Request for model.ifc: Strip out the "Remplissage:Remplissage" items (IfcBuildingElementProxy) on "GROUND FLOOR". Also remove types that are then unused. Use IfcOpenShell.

First a look at what the model holds.

```python
import ifcopenshell
import ifcopenshell.util.element

model = ifcopenshell.open("model.ifc")
print(model.schema)
storey = next(s for s in model.by_type("IfcBuildingStorey") if s.Name == "GROUND FLOOR")
proxies = [e for e in ifcopenshell.util.element.get_decomposition(storey) if e.is_a("IfcBuildingElementProxy")]
seen = {}
for e in proxies:
    element_type = ifcopenshell.util.element.get_type(e)
    name = element_type.Name if element_type not in (None, e) else None
    seen[name] = seen.get(name, 0) + 1
for name, count in sorted(seen.items(), key=str):
    print(count, "x", name)
```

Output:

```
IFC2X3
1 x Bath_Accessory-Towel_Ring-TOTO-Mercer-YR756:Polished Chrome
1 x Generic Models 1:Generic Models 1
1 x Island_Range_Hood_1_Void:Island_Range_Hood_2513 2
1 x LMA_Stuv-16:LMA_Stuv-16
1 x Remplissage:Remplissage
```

```python
import ifcopenshell
import ifcopenshell.api.root
import ifcopenshell.util.element

model = ifcopenshell.open("model.ifc")

storey = next(s for s in model.by_type("IfcBuildingStorey") if s.Name == "GROUND FLOOR")
proxies = [e for e in ifcopenshell.util.element.get_decomposition(storey) if e.is_a("IfcBuildingElementProxy")]
targets = [e for e in proxies if (t := ifcopenshell.util.element.get_type(e)) not in (None, e) and t.Name == "Remplissage:Remplissage"]
types = {ifcopenshell.util.element.get_type(e) for e in targets} - {None, *targets}

for e in targets:
    ifcopenshell.api.root.remove_product(model, product=e)
print(len(targets), "removed")

unused = [t for t in types if not ifcopenshell.util.element.get_types(t)]
for t in unused:
    ifcopenshell.api.root.remove_product(model, product=t)
print(len(unused), "unused types removed")

model.write("model_edited.ifc")
```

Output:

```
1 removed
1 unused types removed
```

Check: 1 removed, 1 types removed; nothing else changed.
